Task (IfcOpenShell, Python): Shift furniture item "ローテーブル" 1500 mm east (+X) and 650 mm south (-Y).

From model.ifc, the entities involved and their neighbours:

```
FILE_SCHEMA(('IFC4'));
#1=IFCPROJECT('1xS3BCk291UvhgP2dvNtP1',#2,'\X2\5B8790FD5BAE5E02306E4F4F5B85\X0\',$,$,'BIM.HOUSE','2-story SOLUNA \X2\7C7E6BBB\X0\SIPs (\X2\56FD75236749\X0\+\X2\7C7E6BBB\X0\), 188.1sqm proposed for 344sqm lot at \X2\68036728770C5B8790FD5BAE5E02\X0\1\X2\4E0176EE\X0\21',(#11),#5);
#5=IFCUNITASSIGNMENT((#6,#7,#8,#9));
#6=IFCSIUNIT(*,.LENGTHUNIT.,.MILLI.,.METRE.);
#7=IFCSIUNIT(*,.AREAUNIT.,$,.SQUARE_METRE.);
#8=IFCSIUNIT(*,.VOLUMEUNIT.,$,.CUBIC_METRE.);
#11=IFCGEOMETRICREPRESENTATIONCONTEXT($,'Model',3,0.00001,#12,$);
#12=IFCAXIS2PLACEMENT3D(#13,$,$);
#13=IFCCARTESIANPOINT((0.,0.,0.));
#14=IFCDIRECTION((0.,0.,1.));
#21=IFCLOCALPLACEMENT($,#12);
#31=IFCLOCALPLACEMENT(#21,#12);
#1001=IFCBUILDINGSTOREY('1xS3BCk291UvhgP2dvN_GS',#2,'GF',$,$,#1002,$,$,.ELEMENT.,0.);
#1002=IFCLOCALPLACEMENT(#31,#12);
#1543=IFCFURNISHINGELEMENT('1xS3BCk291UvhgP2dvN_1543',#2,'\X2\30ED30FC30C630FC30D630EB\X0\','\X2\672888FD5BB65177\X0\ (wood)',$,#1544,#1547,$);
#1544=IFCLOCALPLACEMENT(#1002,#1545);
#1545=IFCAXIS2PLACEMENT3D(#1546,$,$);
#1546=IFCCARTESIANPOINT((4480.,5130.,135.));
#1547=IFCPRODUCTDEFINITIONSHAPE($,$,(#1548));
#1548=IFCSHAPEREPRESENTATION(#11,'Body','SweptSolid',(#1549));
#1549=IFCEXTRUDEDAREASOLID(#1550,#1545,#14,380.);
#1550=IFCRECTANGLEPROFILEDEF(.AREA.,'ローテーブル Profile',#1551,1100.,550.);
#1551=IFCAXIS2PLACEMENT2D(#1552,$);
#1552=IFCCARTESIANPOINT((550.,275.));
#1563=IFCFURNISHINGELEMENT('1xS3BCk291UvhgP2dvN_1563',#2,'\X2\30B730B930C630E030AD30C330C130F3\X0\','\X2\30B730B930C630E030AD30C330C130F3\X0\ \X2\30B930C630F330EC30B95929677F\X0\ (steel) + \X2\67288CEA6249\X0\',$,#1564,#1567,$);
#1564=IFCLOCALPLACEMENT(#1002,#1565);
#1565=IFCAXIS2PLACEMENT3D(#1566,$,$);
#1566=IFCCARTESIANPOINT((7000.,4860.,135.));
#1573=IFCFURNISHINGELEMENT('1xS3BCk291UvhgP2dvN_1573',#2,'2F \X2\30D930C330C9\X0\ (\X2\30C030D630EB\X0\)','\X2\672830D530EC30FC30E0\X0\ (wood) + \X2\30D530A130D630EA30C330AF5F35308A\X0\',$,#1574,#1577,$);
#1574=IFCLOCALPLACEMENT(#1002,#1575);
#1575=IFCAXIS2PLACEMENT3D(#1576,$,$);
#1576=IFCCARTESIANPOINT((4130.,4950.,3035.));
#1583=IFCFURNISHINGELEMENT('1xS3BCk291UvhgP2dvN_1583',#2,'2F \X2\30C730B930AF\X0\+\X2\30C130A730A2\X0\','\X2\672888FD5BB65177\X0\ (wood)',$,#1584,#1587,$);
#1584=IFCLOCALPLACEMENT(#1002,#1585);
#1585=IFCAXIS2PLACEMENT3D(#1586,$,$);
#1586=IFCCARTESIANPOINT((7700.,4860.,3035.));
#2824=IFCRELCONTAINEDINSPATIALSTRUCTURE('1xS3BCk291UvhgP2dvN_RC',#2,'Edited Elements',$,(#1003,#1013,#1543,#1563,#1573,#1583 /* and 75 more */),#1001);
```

```python
import ifcopenshell
import ifcopenshell.api.geometry
import ifcopenshell.util.placement

model = ifcopenshell.open("model.ifc")

item = model.by_guid("1xS3BCk291UvhgP2dvN_1543")
matrix = ifcopenshell.util.placement.get_local_placement(item.ObjectPlacement)
matrix[0, 3] += 1500.0
matrix[1, 3] -= 650.0
ifcopenshell.api.geometry.edit_object_placement(model, product=item, matrix=matrix, is_si=False)

print(ifcopenshell.util.placement.get_local_placement(item.ObjectPlacement).round(3) + 0.0)

model.write("model_rev.ifc")
```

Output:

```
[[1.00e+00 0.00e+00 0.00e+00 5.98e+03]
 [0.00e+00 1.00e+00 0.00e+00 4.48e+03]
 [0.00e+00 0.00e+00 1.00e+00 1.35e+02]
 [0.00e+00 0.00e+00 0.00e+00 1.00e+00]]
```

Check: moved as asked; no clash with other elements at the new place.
